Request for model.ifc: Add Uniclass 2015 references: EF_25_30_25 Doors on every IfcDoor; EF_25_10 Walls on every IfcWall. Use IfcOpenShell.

First a look at what the model holds.

```python
import ifcopenshell

model = ifcopenshell.open("model.ifc")
print(model.schema)
print("classifications:", [c.Name for c in model.by_type("IfcClassification")])
for ifc_class in ("IfcDoor", "IfcRoof", "IfcStair", "IfcWall", "IfcWindow"):
    print(ifc_class, len(model.by_type(ifc_class)))
```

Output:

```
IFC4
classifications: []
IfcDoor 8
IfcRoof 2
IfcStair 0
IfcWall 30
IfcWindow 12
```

```python
import ifcopenshell
import ifcopenshell.api.classification

model = ifcopenshell.open("model.ifc")

system = ifcopenshell.api.classification.add_classification(model, classification="Uniclass 2015")

codes = {
    "IfcDoor": ("EF_25_30_25", "Doors"),
    "IfcWall": ("EF_25_10", "Walls"),
}
for ifc_class, (code, name) in codes.items():
    products = model.by_type(ifc_class)
    ifcopenshell.api.classification.add_reference(
        model, products=products, classification=system, identification=code, name=name
    )
    print(code, len(products))

model.write("model_edited.ifc")
```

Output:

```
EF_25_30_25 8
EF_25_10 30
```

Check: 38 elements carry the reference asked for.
